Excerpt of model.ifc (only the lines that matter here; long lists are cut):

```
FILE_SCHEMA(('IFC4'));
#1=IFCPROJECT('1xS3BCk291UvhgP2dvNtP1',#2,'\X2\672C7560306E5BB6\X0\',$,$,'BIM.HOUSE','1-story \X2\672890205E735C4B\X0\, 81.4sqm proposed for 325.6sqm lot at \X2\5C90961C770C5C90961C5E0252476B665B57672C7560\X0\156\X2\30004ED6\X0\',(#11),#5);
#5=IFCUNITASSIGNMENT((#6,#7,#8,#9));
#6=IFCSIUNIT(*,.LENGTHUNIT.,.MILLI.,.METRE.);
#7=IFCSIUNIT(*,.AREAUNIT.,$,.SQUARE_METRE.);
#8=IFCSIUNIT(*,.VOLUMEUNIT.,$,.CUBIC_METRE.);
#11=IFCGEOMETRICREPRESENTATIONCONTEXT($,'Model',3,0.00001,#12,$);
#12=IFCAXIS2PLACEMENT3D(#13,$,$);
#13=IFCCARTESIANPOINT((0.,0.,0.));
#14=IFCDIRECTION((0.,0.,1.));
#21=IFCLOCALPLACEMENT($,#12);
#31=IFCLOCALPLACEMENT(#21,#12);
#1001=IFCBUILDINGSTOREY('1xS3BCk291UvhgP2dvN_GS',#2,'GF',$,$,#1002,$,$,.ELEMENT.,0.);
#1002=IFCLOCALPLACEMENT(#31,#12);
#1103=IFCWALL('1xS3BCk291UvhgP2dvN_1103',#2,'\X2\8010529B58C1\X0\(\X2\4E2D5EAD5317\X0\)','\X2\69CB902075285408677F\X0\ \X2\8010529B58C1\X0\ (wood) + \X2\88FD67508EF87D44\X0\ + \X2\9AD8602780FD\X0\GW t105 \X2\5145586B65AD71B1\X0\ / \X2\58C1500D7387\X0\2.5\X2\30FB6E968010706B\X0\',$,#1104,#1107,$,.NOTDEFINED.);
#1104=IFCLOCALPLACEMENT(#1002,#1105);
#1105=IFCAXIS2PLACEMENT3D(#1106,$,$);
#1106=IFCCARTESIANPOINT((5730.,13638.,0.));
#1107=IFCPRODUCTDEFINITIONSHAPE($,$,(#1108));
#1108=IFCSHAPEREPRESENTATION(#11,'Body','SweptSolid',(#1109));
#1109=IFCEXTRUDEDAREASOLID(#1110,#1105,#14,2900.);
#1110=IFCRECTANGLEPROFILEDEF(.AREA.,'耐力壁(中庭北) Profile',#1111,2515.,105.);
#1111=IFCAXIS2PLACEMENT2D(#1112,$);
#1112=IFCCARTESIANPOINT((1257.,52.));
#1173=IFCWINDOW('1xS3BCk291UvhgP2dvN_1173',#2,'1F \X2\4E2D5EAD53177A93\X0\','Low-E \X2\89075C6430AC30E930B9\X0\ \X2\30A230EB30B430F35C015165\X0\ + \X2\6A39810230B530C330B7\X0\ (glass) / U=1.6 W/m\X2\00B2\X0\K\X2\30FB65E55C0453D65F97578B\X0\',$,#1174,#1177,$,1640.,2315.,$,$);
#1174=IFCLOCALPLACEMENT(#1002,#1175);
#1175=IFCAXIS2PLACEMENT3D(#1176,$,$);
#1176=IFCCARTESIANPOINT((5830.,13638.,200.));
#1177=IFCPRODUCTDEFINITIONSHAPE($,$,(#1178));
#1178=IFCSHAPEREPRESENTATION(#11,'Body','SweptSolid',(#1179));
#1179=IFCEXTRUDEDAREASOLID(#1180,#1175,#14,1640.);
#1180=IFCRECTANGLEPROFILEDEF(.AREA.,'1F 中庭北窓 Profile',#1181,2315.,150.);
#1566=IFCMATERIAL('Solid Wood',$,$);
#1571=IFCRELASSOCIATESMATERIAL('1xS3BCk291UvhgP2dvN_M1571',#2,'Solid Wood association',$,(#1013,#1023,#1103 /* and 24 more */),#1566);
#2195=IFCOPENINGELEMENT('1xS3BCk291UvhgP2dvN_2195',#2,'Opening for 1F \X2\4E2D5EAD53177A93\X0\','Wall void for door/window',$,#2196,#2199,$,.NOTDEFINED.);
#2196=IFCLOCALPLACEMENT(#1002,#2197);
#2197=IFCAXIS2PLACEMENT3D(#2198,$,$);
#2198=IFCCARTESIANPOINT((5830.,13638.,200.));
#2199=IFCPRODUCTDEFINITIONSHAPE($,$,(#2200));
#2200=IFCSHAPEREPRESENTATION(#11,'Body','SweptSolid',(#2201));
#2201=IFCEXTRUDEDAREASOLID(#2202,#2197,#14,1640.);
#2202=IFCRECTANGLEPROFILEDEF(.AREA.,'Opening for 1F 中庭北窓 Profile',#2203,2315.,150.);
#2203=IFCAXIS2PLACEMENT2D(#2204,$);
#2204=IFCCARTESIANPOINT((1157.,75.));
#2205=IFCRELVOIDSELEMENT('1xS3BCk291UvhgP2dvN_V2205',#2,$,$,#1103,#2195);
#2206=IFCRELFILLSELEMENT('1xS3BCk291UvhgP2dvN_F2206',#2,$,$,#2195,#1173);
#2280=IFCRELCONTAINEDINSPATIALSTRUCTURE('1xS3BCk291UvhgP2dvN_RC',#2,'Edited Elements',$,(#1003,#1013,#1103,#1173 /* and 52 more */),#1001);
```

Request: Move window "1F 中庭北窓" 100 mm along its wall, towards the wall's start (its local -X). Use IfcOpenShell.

```python
import ifcopenshell
import ifcopenshell.api.geometry
import ifcopenshell.util.placement

model = ifcopenshell.open("model.ifc")

window = model.by_id(1173)
opening = window.FillsVoids[0].RelatingOpeningElement
wall = opening.VoidsElements[0].RelatingBuildingElement

wall_matrix = ifcopenshell.util.placement.get_local_placement(wall.ObjectPlacement)
shift = wall_matrix[:3, 0] * -100.0
before = ifcopenshell.util.placement.get_local_placement(window.ObjectPlacement)[:3, 3].copy()

# The window is not placed relative to its opening, so move both.
for product in (opening, window):
    matrix = ifcopenshell.util.placement.get_local_placement(product.ObjectPlacement)
    matrix[:3, 3] += shift
    ifcopenshell.api.geometry.edit_object_placement(model, product=product, matrix=matrix, is_si=False)

after = ifcopenshell.util.placement.get_local_placement(window.ObjectPlacement)[:3, 3]
print("window moved by", (after - before).round(3) + 0.0)

model.write("model_updated.ifc")
```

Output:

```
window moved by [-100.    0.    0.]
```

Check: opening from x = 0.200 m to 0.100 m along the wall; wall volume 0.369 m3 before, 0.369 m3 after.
